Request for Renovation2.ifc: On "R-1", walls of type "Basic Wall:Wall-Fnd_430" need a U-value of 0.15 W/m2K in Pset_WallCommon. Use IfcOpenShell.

First a look at what the model holds.

```python
import ifcopenshell
import ifcopenshell.util.element

model = ifcopenshell.open("Renovation2.ifc")
print(model.schema)
storey = next(s for s in model.by_type("IfcBuildingStorey") if s.Name == "R-1")
walls = [e for e in ifcopenshell.util.element.get_decomposition(storey) if e.is_a("IfcWall")]
seen = {}
for e in walls:
    element_type = ifcopenshell.util.element.get_type(e)
    key = (element_type.Name if element_type != e and element_type else None, ifcopenshell.util.element.get_pset(e, "Pset_WallCommon", "ThermalTransmittance"))
    seen[key] = seen.get(key, 0) + 1
for (name, value), count in sorted(seen.items(), key=str):
    print(count, "x", name, "|", value)
```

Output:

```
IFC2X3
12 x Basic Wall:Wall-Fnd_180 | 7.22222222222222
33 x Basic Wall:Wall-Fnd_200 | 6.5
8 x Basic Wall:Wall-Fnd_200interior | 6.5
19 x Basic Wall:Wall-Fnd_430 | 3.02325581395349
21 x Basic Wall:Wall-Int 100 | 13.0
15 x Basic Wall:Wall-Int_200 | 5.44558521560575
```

```python
import ifcopenshell
import ifcopenshell.api.pset
import ifcopenshell.util.element

model = ifcopenshell.open("Renovation2.ifc")

storey = next(s for s in model.by_type("IfcBuildingStorey") if s.Name == "R-1")
walls = [e for e in ifcopenshell.util.element.get_decomposition(storey) if e.is_a("IfcWall")]

count = 0
for e in walls:
    element_type = ifcopenshell.util.element.get_type(e)
    if element_type in (None, e) or element_type.Name != "Basic Wall:Wall-Fnd_430":
        continue
    # add_pset returns the element's existing set when there is one.
    pset = ifcopenshell.api.pset.add_pset(model, product=e, name="Pset_WallCommon")
    ifcopenshell.api.pset.edit_pset(model, pset=pset, properties={"ThermalTransmittance": 0.15})
    count += 1

print(count, "walls updated")

model.write("Renovation2_rev.ifc")
```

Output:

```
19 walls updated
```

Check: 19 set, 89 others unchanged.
